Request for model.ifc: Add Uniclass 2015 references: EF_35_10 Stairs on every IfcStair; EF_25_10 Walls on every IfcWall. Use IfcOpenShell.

First a look at what the model holds.

```python
import ifcopenshell

model = ifcopenshell.open("model.ifc")
print(model.schema)
print("classifications:", [c.Name for c in model.by_type("IfcClassification")])
for ifc_class in ("IfcDoor", "IfcRoof", "IfcStair", "IfcWall", "IfcWindow"):
    print(ifc_class, len(model.by_type(ifc_class)))
```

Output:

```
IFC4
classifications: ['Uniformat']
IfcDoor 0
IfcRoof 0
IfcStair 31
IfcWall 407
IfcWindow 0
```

```python
import ifcopenshell
import ifcopenshell.api.classification

model = ifcopenshell.open("model.ifc")

system = ifcopenshell.api.classification.add_classification(model, classification="Uniclass 2015")

codes = {
    "IfcStair": ("EF_35_10", "Stairs"),
    "IfcWall": ("EF_25_10", "Walls"),
}
for ifc_class, (code, name) in codes.items():
    products = model.by_type(ifc_class)
    ifcopenshell.api.classification.add_reference(
        model, products=products, classification=system, identification=code, name=name
    )
    print(code, len(products))

model.write("model_edited.ifc")
```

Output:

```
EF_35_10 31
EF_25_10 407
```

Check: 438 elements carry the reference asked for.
